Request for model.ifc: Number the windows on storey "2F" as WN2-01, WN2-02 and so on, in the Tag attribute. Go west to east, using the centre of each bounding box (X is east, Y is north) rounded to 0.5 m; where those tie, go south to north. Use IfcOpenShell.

First a look at what the model holds.

```python
import ifcopenshell
import ifcopenshell.util.element
import ifcopenshell.util.placement

model = ifcopenshell.open("model.ifc")
print(model.schema)
storey = next(s for s in model.by_type("IfcBuildingStorey") if s.Name == "2F")
windows = [e for e in ifcopenshell.util.element.get_decomposition(storey) if e.is_a("IfcWindow")]
for e in sorted(windows, key=lambda e: e.id()):
    origin = ifcopenshell.util.placement.get_local_placement(e.ObjectPlacement)[:3, 3]
    print(e.id(), e.Tag, e.Name, origin.round(2) + 0.0, sep=" | ")
```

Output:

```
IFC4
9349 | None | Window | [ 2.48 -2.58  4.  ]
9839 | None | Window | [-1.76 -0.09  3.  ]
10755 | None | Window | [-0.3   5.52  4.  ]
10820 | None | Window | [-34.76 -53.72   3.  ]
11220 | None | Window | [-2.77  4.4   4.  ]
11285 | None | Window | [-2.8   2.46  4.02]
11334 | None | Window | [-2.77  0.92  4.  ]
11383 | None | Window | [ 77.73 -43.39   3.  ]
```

```python
import ifcopenshell
import ifcopenshell.geom
import ifcopenshell.util.element
import ifcopenshell.util.shape

model = ifcopenshell.open("model.ifc")
settings = ifcopenshell.geom.settings()
settings.set("use-world-coords", True)


def centre(element):
    shape = ifcopenshell.geom.create_shape(settings, element)
    return ifcopenshell.util.shape.get_bbox_centroid(shape.geometry)


storey = next(s for s in model.by_type("IfcBuildingStorey") if s.Name == "2F")
windows = [e for e in ifcopenshell.util.element.get_decomposition(storey) if e.is_a("IfcWindow")]

# Insertion points can sit at a corner or the storey origin, so sort by the geometry (in metres).
centres = {e: centre(e) for e in windows}
windows.sort(key=lambda e: (round(centres[e][0] / 0.5), centres[e][1]))

for i, e in enumerate(windows, start=1):
    number = f"WN2-{i:02d}"
    e.Tag = number
    print(e.id(), number)

model.write("model_updated.ifc")
```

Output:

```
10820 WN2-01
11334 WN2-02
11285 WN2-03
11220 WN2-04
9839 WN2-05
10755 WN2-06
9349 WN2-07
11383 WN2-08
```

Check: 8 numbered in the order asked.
